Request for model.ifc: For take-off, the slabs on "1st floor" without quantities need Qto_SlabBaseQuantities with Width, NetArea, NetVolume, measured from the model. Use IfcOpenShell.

First a look at what the model holds.

```python
import ifcopenshell
import ifcopenshell.util.element
import ifcopenshell.util.unit

model = ifcopenshell.open("model.ifc")
print(model.schema)
for unit_type in ("LENGTHUNIT", "AREAUNIT", "VOLUMEUNIT"):
    print(unit_type, ifcopenshell.util.unit.calculate_unit_scale(model, unit_type))
storey = next(s for s in model.by_type("IfcBuildingStorey") if s.Name == "1st floor")
slabs = [e for e in ifcopenshell.util.element.get_decomposition(storey) if e.is_a("IfcSlab")]
for e in sorted(slabs, key=lambda e: e.id()):
    print(e.id(), e.is_a(), e.Name, list(ifcopenshell.util.element.get_psets(e, qtos_only=True)), sep=" | ")
```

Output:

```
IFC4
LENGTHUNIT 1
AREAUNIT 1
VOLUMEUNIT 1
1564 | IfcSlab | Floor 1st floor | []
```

```python
import ifcopenshell
import ifcopenshell.api.pset
import ifcopenshell.geom
import ifcopenshell.util.element
import ifcopenshell.util.shape
import ifcopenshell.util.unit

model = ifcopenshell.open("model.ifc")
unit_scale = ifcopenshell.util.unit.calculate_unit_scale(model)
area_scale = ifcopenshell.util.unit.calculate_unit_scale(model, "AREAUNIT")
volume_scale = ifcopenshell.util.unit.calculate_unit_scale(model, "VOLUMEUNIT")
settings = ifcopenshell.geom.settings()

storey = next(s for s in model.by_type("IfcBuildingStorey") if s.Name == "1st floor")
slabs = [e for e in ifcopenshell.util.element.get_decomposition(storey) if e.is_a("IfcSlab")]

for e in sorted(slabs, key=lambda e: e.id()):
    if ifcopenshell.util.element.get_psets(e, qtos_only=True, should_inherit=False):
        continue
    # Geometry comes back in metres, in the element's own axes.
    shape = ifcopenshell.geom.create_shape(settings, e)
    values = {
        "Width": ifcopenshell.util.shape.get_z(shape.geometry) / unit_scale,
        "NetArea": ifcopenshell.util.shape.get_footprint_area(shape.geometry) / area_scale,
        "NetVolume": ifcopenshell.util.shape.get_volume(shape.geometry) / volume_scale,
    }
    qto = ifcopenshell.api.pset.add_qto(model, product=e, name="Qto_SlabBaseQuantities")
    ifcopenshell.api.pset.edit_qto(model, qto=qto, properties=values)
    print(e.id(), {k: round(v, 3) for k, v in values.items()})

model.write("model_edited.ifc")
```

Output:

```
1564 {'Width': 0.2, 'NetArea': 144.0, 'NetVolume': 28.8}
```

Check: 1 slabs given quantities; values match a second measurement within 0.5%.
